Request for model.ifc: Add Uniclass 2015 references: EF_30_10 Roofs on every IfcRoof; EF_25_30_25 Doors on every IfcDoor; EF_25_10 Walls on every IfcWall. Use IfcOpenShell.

First a look at what the model holds.

```python
import ifcopenshell

model = ifcopenshell.open("model.ifc")
print(model.schema)
print("classifications:", [c.Name for c in model.by_type("IfcClassification")])
for ifc_class in ("IfcDoor", "IfcRoof", "IfcStair", "IfcWall", "IfcWindow"):
    print(ifc_class, len(model.by_type(ifc_class)))
```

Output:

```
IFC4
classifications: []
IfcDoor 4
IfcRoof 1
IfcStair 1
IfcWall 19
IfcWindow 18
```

```python
import ifcopenshell
import ifcopenshell.api.classification

model = ifcopenshell.open("model.ifc")

system = ifcopenshell.api.classification.add_classification(model, classification="Uniclass 2015")

codes = {
    "IfcRoof": ("EF_30_10", "Roofs"),
    "IfcDoor": ("EF_25_30_25", "Doors"),
    "IfcWall": ("EF_25_10", "Walls"),
}
for ifc_class, (code, name) in codes.items():
    products = model.by_type(ifc_class)
    ifcopenshell.api.classification.add_reference(
        model, products=products, classification=system, identification=code, name=name
    )
    print(code, len(products))

model.write("model_updated.ifc")
```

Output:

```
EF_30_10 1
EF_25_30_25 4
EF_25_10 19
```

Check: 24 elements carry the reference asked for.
